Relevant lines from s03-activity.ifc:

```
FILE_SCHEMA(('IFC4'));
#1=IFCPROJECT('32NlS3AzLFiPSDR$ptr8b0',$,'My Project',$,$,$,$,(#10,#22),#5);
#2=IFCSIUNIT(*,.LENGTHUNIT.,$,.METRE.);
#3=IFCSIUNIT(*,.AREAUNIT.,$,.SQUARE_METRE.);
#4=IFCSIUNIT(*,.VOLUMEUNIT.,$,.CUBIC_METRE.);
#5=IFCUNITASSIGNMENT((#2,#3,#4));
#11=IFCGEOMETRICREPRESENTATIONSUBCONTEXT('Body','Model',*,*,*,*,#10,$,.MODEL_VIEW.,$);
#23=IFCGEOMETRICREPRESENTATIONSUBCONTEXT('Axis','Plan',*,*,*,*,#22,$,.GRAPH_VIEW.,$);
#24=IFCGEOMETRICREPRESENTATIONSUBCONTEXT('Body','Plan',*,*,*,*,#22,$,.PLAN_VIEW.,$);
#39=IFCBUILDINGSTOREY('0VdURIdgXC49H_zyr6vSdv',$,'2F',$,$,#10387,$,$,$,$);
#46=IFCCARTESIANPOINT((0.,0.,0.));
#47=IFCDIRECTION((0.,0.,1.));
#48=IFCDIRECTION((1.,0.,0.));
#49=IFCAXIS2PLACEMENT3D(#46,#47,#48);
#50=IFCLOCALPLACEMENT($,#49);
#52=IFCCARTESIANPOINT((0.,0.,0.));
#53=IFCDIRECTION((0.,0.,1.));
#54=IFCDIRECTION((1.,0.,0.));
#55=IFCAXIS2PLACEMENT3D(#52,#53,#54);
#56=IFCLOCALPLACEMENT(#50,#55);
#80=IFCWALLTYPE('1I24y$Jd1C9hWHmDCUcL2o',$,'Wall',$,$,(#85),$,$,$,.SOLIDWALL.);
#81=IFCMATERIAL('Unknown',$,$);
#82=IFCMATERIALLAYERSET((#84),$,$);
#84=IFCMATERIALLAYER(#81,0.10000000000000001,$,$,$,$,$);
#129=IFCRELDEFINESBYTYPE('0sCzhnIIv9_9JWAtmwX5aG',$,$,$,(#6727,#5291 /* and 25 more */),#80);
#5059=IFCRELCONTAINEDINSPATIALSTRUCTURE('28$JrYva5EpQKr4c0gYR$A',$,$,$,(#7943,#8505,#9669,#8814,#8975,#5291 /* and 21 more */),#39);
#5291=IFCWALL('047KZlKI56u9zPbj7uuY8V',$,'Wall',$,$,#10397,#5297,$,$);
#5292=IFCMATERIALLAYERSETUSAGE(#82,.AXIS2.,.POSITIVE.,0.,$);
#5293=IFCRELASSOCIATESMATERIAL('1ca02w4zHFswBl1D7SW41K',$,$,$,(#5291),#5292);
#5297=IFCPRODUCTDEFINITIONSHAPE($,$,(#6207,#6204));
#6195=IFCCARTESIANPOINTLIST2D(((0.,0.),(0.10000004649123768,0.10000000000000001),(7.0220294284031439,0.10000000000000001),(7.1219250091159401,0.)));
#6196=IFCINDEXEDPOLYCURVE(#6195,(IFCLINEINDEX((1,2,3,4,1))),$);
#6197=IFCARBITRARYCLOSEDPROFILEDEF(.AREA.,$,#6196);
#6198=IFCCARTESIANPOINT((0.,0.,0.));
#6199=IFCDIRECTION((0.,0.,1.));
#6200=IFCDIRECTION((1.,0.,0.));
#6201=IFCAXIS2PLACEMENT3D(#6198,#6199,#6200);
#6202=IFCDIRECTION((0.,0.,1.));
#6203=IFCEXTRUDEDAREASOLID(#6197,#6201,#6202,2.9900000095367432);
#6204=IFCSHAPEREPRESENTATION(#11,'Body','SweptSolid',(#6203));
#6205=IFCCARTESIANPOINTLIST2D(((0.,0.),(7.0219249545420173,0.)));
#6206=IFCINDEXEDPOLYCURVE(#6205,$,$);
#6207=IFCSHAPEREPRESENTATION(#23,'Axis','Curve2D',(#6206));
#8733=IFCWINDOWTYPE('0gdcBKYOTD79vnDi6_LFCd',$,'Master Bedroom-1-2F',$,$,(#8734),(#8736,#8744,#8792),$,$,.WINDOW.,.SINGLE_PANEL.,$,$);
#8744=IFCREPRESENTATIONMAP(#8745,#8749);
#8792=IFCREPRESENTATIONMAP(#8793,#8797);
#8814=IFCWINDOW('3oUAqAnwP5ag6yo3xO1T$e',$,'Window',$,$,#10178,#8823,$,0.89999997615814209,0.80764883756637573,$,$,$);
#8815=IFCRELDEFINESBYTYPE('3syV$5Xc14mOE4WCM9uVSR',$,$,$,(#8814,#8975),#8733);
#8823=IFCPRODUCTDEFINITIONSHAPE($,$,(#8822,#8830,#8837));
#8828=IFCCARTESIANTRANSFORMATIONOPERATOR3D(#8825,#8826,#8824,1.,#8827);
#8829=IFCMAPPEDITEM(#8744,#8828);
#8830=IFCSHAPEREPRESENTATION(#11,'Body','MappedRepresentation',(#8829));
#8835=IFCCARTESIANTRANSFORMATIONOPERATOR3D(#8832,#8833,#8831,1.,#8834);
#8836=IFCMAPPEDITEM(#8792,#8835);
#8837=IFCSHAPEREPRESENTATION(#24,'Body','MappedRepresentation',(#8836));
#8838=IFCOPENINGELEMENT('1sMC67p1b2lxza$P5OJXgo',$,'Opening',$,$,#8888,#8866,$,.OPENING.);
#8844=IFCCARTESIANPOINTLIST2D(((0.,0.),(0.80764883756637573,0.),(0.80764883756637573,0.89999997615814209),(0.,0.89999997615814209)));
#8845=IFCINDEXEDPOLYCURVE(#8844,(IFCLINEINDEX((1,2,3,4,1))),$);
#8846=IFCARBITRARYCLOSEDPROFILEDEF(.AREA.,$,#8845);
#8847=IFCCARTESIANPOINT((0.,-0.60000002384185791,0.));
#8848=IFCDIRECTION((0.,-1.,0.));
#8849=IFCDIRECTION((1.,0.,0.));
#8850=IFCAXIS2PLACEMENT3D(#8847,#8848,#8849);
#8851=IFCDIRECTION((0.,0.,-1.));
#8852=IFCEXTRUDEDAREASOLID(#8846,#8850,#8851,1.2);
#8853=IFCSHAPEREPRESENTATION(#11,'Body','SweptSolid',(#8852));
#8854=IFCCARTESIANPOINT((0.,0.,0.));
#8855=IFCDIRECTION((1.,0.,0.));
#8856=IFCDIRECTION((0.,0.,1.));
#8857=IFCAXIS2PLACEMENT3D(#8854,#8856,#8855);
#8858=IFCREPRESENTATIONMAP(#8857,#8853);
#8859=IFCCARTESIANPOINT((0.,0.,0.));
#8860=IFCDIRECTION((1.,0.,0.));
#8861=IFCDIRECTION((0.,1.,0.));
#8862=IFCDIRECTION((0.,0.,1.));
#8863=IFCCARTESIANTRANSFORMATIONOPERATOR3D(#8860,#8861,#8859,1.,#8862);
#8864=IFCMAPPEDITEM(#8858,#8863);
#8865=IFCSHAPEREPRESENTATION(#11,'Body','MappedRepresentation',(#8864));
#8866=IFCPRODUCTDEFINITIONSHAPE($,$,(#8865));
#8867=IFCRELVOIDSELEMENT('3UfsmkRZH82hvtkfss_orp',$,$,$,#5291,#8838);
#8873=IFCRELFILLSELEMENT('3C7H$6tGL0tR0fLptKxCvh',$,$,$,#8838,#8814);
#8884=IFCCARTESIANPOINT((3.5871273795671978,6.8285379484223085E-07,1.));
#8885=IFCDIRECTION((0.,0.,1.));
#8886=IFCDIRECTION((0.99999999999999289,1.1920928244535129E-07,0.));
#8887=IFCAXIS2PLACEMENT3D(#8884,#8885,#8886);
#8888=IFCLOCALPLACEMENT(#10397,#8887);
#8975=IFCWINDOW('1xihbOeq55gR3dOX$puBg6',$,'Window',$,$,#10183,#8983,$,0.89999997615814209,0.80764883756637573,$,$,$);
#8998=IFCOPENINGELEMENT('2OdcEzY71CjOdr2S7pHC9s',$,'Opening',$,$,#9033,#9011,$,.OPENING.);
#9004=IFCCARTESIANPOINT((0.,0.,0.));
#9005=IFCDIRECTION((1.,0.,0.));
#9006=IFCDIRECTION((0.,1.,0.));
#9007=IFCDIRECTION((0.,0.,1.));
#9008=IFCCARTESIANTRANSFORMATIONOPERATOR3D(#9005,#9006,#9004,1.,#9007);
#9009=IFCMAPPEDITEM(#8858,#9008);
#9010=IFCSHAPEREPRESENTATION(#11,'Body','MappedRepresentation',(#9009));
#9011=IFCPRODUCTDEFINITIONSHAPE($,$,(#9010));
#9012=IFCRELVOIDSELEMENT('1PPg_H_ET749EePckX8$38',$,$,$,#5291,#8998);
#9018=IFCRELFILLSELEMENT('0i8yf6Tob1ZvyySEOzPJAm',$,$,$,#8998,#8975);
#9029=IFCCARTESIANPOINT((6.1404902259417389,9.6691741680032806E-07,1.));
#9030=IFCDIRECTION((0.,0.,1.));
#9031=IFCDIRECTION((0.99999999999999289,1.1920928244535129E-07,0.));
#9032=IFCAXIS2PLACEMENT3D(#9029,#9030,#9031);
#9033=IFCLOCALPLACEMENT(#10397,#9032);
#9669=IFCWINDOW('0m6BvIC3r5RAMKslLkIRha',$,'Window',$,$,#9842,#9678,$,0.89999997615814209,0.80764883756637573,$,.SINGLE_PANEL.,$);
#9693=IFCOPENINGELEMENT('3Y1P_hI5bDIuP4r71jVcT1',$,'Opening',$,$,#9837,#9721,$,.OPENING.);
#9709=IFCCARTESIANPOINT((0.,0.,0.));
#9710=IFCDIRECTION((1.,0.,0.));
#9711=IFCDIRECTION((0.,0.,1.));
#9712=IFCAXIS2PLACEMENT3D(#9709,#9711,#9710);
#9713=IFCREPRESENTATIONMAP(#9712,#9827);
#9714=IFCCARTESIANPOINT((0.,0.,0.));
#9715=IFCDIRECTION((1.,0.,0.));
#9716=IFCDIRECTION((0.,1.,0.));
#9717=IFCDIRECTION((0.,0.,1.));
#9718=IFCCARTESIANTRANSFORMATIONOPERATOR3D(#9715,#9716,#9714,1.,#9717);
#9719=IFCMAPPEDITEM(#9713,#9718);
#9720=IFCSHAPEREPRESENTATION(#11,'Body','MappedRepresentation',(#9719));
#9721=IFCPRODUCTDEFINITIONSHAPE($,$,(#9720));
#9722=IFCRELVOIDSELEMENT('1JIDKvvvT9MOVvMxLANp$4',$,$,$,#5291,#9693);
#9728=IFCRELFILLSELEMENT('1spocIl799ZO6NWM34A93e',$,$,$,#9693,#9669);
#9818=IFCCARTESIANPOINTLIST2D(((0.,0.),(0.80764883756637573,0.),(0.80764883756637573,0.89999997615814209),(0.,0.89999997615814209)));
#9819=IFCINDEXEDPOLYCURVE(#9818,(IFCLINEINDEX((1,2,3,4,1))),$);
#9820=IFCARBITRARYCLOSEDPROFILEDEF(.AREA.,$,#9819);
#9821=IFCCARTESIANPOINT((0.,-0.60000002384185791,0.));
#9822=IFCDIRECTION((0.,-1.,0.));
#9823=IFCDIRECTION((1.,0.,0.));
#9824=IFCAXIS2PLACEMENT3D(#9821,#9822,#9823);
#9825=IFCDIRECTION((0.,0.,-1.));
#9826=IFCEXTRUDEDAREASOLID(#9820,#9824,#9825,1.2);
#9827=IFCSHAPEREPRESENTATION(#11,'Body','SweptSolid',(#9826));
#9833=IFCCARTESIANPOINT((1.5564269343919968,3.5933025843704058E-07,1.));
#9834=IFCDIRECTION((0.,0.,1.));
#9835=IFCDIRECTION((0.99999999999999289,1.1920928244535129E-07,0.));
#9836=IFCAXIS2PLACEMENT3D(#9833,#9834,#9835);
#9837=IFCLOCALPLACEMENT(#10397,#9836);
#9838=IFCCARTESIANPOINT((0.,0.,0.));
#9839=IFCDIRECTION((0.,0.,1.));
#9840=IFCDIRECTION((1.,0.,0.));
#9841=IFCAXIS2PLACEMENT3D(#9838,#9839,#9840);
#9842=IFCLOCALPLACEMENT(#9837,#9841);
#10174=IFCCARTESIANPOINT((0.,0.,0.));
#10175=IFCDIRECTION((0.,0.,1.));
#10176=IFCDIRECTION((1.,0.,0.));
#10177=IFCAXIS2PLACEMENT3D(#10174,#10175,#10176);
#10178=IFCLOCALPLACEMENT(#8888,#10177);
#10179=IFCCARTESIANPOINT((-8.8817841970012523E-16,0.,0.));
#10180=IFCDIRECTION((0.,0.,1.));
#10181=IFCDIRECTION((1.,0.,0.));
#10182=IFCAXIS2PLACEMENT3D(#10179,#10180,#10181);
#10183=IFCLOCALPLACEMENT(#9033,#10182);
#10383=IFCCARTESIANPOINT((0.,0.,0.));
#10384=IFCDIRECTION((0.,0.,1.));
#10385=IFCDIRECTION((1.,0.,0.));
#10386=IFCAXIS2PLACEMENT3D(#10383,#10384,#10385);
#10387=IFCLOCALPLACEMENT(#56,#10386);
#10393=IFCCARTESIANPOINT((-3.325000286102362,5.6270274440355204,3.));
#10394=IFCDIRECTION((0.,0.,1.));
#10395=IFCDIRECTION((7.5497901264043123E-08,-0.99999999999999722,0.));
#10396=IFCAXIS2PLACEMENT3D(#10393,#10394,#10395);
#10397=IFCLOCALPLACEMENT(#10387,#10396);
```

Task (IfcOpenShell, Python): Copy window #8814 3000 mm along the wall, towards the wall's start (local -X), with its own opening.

```python
import ifcopenshell
import ifcopenshell.api.feature
import ifcopenshell.api.geometry
import ifcopenshell.api.root
import ifcopenshell.geom
import ifcopenshell.util.element
import ifcopenshell.util.placement
import ifcopenshell.util.shape

model = ifcopenshell.open("s03-activity.ifc")
settings = ifcopenshell.geom.settings()


def volume(element):
    """Net volume in cubic metres, openings subtracted."""
    shape = ifcopenshell.geom.create_shape(settings, element)
    return ifcopenshell.util.shape.get_volume(shape.geometry)


window = model.by_guid("3oUAqAnwP5ag6yo3xO1T$e")
opening = window.FillsVoids[0].RelatingOpeningElement
wall = opening.VoidsElements[0].RelatingBuildingElement
before = volume(wall)
shift = ifcopenshell.util.placement.get_local_placement(wall.ObjectPlacement)[:3, 0] * -3.0

# copy_class copies the void relationship, type, container and properties, but no geometry.
new_opening = ifcopenshell.api.root.copy_class(model, product=opening)
new_opening.Representation = ifcopenshell.util.element.copy_deep(
    model, opening.Representation, exclude=["IfcGeometricRepresentationContext", "IfcRepresentationMap"]
)
new_window = ifcopenshell.api.root.copy_class(model, product=window)
new_window.Representation = ifcopenshell.util.element.copy_deep(
    model, window.Representation, exclude=["IfcGeometricRepresentationContext", "IfcRepresentationMap"]
)
ifcopenshell.api.feature.add_filling(model, opening=new_opening, element=new_window)

for old, new in ((opening, new_opening), (window, new_window)):
    matrix = ifcopenshell.util.placement.get_local_placement(old.ObjectPlacement)
    matrix[:3, 3] += shift
    ifcopenshell.api.geometry.edit_object_placement(model, product=new, matrix=matrix, is_si=False)

after = volume(wall)

print(f"wall volume {before:.3f} -> {after:.3f} m3")

model.write("s03-activity_rev.ifc")
```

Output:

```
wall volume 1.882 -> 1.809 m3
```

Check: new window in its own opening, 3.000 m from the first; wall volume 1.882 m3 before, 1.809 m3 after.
